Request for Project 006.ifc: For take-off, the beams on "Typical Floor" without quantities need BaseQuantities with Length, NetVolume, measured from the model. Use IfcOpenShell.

First a look at what the model holds.

```python
import ifcopenshell
import ifcopenshell.util.element
import ifcopenshell.util.unit

model = ifcopenshell.open("Project 006.ifc")
print(model.schema)
for unit_type in ("LENGTHUNIT", "AREAUNIT", "VOLUMEUNIT"):
    print(unit_type, ifcopenshell.util.unit.calculate_unit_scale(model, unit_type))
storey = next(s for s in model.by_type("IfcBuildingStorey") if s.Name == "Typical Floor")
beams = [e for e in ifcopenshell.util.element.get_decomposition(storey) if e.is_a("IfcBeam")]
for e in sorted(beams, key=lambda e: e.id()):
    print(e.id(), e.is_a(), e.Name, list(ifcopenshell.util.element.get_psets(e, qtos_only=True)), sep=" | ")
```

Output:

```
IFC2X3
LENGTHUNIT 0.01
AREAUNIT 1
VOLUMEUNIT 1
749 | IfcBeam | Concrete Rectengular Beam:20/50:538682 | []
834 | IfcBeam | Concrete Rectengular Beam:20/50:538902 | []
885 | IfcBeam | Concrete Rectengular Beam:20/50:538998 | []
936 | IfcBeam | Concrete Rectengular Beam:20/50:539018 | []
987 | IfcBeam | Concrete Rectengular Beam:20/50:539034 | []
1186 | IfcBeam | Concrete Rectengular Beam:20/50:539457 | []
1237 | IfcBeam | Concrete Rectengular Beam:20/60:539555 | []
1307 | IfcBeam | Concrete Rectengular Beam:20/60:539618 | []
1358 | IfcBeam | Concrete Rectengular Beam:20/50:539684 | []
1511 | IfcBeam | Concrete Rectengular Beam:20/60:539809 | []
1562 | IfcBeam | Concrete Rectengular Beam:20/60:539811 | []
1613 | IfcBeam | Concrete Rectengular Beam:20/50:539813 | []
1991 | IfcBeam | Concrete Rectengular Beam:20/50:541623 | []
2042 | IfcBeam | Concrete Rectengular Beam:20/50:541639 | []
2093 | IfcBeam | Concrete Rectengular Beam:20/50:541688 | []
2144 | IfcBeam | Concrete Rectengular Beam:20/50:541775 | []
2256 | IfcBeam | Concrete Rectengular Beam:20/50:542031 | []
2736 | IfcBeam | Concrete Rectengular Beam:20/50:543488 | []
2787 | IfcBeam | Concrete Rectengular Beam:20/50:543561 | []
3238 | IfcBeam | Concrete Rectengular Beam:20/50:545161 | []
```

```python
import ifcopenshell
import ifcopenshell.api.pset
import ifcopenshell.geom
import ifcopenshell.util.element
import ifcopenshell.util.shape
import ifcopenshell.util.unit

model = ifcopenshell.open("Project 006.ifc")
unit_scale = ifcopenshell.util.unit.calculate_unit_scale(model)
volume_scale = ifcopenshell.util.unit.calculate_unit_scale(model, "VOLUMEUNIT")
settings = ifcopenshell.geom.settings()

storey = next(s for s in model.by_type("IfcBuildingStorey") if s.Name == "Typical Floor")
beams = [e for e in ifcopenshell.util.element.get_decomposition(storey) if e.is_a("IfcBeam")]

for e in sorted(beams, key=lambda e: e.id()):
    if ifcopenshell.util.element.get_psets(e, qtos_only=True, should_inherit=False):
        continue
    # Geometry comes back in metres, in the element's own axes.
    shape = ifcopenshell.geom.create_shape(settings, e)
    values = {
        "Length": ifcopenshell.util.shape.get_max_xyz(shape.geometry) / unit_scale,
        "NetVolume": ifcopenshell.util.shape.get_volume(shape.geometry) / volume_scale,
    }
    qto = ifcopenshell.api.pset.add_qto(model, product=e, name="BaseQuantities")
    ifcopenshell.api.pset.edit_qto(model, qto=qto, properties=values)
    print(e.id(), {k: round(v, 3) for k, v in values.items()})

model.write("Project 006_v2.ifc")
```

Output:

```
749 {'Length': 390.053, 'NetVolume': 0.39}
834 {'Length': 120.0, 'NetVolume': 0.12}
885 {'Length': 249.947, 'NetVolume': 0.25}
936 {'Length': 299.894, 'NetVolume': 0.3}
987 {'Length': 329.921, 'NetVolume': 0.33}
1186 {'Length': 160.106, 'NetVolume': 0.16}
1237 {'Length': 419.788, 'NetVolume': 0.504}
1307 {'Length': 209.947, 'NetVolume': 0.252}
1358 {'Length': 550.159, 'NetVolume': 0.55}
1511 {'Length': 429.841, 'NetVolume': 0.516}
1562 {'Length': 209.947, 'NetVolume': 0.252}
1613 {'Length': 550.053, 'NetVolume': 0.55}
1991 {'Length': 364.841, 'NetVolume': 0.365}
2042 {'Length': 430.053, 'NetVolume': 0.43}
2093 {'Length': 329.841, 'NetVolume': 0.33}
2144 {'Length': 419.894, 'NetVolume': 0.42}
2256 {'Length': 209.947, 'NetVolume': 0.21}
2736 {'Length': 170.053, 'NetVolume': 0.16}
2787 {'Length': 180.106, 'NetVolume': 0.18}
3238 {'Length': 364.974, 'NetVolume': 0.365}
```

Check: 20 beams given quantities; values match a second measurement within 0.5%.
